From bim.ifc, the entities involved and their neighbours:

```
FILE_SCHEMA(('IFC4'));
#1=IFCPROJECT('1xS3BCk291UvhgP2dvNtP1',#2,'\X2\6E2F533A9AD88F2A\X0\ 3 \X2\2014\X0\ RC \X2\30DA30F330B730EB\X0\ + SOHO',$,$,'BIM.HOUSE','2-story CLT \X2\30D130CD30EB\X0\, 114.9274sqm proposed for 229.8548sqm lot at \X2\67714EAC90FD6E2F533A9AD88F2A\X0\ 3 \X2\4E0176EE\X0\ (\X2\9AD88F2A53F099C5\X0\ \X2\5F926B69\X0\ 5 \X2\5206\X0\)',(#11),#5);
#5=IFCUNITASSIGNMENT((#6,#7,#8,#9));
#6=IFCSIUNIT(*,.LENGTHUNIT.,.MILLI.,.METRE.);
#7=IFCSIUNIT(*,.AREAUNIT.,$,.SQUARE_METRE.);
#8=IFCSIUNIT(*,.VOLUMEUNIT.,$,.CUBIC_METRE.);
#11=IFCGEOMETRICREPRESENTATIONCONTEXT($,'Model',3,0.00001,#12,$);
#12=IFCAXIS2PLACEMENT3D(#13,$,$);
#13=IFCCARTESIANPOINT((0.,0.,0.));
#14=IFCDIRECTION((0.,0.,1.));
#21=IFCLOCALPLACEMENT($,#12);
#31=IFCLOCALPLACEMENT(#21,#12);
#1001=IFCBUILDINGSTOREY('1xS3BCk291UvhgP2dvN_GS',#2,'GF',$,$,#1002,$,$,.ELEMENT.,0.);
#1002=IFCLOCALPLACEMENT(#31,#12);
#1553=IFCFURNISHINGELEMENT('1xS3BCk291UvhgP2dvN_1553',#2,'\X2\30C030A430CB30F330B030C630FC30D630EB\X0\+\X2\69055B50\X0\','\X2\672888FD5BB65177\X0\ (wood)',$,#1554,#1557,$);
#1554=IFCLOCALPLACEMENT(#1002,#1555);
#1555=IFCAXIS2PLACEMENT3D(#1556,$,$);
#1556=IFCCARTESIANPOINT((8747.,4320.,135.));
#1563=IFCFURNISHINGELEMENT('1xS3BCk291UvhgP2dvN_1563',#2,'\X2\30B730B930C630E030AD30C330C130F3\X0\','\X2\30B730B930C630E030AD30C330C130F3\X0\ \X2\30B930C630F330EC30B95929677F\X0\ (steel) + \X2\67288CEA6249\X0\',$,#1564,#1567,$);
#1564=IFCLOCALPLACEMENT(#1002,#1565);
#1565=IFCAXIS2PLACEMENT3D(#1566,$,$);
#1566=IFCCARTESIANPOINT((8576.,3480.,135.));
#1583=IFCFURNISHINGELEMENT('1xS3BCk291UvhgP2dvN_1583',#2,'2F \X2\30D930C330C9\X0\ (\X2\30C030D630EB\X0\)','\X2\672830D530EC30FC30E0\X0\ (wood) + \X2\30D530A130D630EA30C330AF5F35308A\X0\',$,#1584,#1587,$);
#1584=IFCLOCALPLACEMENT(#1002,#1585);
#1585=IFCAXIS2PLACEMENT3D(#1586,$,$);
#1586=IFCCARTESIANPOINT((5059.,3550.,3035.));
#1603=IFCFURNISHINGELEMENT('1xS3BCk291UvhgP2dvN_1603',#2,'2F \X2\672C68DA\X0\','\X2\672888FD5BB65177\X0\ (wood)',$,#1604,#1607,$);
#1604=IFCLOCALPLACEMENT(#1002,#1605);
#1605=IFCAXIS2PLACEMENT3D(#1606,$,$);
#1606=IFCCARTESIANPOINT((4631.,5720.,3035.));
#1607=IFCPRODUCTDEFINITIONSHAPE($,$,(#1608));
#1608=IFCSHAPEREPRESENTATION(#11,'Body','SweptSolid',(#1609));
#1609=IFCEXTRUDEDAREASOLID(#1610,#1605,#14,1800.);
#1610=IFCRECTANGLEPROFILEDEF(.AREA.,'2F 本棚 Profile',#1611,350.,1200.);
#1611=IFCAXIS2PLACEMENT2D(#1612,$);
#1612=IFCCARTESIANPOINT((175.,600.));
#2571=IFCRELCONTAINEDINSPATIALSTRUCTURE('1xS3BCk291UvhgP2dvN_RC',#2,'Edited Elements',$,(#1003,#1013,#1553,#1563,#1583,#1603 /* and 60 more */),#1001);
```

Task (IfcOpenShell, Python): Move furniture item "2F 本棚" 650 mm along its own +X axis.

```python
import ifcopenshell
import ifcopenshell.api.geometry
import ifcopenshell.util.placement
import ifcopenshell.util.unit

model = ifcopenshell.open("bim.ifc")
unit_scale = ifcopenshell.util.unit.calculate_unit_scale(model)

item = model.by_guid("1xS3BCk291UvhgP2dvN_1603")
matrix = ifcopenshell.util.placement.get_local_placement(item.ObjectPlacement)
matrix[:3, 3] += matrix[:3, 0] * 0.65 / unit_scale
ifcopenshell.api.geometry.edit_object_placement(model, product=item, matrix=matrix, is_si=False)

print(ifcopenshell.util.placement.get_local_placement(item.ObjectPlacement).round(3) + 0.0)

model.write("bim_updated.ifc")
```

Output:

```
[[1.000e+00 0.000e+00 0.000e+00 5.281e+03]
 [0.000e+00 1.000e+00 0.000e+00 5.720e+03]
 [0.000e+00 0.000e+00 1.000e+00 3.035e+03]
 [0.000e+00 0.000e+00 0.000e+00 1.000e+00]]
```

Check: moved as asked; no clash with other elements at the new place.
